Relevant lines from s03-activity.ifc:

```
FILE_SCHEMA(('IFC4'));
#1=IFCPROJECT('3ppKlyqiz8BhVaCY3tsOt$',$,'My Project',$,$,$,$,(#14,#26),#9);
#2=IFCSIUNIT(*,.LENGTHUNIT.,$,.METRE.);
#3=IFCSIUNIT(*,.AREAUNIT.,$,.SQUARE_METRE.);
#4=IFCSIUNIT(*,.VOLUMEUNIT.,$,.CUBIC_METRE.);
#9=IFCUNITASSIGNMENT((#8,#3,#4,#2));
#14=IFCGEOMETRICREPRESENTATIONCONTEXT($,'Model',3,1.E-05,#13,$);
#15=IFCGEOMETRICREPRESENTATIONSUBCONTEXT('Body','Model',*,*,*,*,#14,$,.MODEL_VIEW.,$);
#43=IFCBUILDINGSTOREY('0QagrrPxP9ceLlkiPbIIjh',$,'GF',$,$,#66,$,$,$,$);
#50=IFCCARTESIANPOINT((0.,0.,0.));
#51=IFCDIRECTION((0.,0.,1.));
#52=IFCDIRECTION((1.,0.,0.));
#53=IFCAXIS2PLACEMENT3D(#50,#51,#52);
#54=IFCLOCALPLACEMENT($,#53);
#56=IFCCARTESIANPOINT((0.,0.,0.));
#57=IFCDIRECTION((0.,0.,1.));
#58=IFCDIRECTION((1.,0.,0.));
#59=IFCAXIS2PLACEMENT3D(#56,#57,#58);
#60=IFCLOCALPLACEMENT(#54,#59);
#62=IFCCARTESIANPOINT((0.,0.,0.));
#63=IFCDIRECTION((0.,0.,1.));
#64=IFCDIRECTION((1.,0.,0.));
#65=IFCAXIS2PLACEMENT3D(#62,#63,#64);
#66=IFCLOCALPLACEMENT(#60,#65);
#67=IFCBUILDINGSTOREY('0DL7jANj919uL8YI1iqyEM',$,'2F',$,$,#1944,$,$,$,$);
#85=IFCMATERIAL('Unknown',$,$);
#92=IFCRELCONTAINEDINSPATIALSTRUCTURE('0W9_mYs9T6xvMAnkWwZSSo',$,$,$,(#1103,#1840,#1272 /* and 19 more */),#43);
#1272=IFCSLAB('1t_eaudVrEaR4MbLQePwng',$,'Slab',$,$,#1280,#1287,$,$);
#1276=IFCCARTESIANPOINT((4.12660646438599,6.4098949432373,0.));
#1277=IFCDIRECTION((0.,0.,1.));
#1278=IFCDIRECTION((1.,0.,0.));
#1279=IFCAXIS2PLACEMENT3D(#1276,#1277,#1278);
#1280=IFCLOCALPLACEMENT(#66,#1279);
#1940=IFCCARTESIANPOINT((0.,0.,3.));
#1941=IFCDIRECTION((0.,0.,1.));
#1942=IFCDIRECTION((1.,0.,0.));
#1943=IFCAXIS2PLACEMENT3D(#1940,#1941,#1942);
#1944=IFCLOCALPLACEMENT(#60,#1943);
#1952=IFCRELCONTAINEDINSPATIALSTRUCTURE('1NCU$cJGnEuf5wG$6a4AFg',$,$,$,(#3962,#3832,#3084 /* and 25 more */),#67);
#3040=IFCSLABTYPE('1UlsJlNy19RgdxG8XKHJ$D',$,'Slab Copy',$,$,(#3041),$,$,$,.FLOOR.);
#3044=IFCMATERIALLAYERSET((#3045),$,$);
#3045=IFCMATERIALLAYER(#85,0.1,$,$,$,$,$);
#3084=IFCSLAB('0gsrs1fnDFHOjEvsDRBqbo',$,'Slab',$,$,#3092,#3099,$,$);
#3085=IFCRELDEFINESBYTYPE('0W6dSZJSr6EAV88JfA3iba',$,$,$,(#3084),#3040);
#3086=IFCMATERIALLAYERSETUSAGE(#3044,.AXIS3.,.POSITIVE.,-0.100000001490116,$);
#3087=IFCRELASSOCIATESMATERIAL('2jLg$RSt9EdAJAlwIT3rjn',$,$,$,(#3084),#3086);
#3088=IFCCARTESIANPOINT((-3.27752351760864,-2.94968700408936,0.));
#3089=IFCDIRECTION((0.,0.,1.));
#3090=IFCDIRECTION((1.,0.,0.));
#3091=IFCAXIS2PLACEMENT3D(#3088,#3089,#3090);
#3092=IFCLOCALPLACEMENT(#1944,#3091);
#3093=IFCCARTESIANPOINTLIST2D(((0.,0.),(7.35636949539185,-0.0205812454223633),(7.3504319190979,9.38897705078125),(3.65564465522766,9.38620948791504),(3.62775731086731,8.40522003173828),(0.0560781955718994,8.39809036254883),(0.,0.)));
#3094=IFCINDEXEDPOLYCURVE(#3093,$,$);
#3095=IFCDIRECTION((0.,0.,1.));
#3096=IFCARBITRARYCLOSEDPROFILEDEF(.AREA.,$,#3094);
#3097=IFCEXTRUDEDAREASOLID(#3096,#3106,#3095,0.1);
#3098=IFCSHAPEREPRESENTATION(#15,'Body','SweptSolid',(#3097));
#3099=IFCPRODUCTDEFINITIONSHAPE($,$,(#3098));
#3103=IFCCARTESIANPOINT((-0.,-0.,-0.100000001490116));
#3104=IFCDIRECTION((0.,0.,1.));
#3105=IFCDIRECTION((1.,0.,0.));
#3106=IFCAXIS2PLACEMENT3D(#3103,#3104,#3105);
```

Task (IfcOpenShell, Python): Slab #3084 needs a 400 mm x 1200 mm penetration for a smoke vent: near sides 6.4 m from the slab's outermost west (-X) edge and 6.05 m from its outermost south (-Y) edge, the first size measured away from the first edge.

```python
import numpy as np
import ifcopenshell
import ifcopenshell.api.feature
import ifcopenshell.api.geometry
import ifcopenshell.api.root
import ifcopenshell.geom
import ifcopenshell.util.placement
import ifcopenshell.util.representation
import ifcopenshell.util.shape
import ifcopenshell.util.unit

model = ifcopenshell.open("s03-activity.ifc")
unit_scale = ifcopenshell.util.unit.calculate_unit_scale(model)
settings = ifcopenshell.geom.settings()


def volume(element):
    """Net volume in cubic metres, openings subtracted."""
    shape = ifcopenshell.geom.create_shape(settings, element)
    return ifcopenshell.util.shape.get_volume(shape.geometry)


slab = model.by_id(3084)
before = volume(slab)

# Extent in the slab's own axes, in metres. The edges named are its -X and -Y sides.
slab_shape = ifcopenshell.geom.create_shape(settings, slab)
vertices = ifcopenshell.util.shape.get_vertices(slab_shape.geometry)
x_min, y_min, bottom = vertices.min(axis=0)
top = vertices[:, 2].max()

opening = ifcopenshell.api.root.create_entity(model, ifc_class="IfcOpeningElement", name="Smoke vent opening", predefined_type="OPENING")
context = ifcopenshell.util.representation.get_context(model, "Model", "Body", "MODEL_VIEW")
width, depth = 0.4, 1.2
outline = [(0.0, 0.0), (width, 0.0), (width, depth), (0.0, depth), (0.0, 0.0)]
# Overshoot both faces by 50 mm so the cut is clean.
shape = ifcopenshell.api.geometry.add_slab_representation(
    model, context=context, depth=top - bottom + 0.1, polyline=outline
)
ifcopenshell.api.geometry.assign_representation(model, product=opening, representation=shape)

matrix = ifcopenshell.util.placement.get_local_placement(slab.ObjectPlacement)
matrix[:, 3] = matrix @ np.append(np.array([x_min + 6.4, y_min + 6.05, bottom - 0.05]) / unit_scale, 1.0)
ifcopenshell.api.geometry.edit_object_placement(model, product=opening, matrix=matrix, is_si=False)
ifcopenshell.api.feature.add_feature(model, feature=opening, element=slab)

after = volume(slab)

print(f"slab volume {before:.3f} -> {after:.3f} m3")

model.write("s03-activity_updated.ifc")
```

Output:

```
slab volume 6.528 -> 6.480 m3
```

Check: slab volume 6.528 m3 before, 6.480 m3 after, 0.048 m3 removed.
